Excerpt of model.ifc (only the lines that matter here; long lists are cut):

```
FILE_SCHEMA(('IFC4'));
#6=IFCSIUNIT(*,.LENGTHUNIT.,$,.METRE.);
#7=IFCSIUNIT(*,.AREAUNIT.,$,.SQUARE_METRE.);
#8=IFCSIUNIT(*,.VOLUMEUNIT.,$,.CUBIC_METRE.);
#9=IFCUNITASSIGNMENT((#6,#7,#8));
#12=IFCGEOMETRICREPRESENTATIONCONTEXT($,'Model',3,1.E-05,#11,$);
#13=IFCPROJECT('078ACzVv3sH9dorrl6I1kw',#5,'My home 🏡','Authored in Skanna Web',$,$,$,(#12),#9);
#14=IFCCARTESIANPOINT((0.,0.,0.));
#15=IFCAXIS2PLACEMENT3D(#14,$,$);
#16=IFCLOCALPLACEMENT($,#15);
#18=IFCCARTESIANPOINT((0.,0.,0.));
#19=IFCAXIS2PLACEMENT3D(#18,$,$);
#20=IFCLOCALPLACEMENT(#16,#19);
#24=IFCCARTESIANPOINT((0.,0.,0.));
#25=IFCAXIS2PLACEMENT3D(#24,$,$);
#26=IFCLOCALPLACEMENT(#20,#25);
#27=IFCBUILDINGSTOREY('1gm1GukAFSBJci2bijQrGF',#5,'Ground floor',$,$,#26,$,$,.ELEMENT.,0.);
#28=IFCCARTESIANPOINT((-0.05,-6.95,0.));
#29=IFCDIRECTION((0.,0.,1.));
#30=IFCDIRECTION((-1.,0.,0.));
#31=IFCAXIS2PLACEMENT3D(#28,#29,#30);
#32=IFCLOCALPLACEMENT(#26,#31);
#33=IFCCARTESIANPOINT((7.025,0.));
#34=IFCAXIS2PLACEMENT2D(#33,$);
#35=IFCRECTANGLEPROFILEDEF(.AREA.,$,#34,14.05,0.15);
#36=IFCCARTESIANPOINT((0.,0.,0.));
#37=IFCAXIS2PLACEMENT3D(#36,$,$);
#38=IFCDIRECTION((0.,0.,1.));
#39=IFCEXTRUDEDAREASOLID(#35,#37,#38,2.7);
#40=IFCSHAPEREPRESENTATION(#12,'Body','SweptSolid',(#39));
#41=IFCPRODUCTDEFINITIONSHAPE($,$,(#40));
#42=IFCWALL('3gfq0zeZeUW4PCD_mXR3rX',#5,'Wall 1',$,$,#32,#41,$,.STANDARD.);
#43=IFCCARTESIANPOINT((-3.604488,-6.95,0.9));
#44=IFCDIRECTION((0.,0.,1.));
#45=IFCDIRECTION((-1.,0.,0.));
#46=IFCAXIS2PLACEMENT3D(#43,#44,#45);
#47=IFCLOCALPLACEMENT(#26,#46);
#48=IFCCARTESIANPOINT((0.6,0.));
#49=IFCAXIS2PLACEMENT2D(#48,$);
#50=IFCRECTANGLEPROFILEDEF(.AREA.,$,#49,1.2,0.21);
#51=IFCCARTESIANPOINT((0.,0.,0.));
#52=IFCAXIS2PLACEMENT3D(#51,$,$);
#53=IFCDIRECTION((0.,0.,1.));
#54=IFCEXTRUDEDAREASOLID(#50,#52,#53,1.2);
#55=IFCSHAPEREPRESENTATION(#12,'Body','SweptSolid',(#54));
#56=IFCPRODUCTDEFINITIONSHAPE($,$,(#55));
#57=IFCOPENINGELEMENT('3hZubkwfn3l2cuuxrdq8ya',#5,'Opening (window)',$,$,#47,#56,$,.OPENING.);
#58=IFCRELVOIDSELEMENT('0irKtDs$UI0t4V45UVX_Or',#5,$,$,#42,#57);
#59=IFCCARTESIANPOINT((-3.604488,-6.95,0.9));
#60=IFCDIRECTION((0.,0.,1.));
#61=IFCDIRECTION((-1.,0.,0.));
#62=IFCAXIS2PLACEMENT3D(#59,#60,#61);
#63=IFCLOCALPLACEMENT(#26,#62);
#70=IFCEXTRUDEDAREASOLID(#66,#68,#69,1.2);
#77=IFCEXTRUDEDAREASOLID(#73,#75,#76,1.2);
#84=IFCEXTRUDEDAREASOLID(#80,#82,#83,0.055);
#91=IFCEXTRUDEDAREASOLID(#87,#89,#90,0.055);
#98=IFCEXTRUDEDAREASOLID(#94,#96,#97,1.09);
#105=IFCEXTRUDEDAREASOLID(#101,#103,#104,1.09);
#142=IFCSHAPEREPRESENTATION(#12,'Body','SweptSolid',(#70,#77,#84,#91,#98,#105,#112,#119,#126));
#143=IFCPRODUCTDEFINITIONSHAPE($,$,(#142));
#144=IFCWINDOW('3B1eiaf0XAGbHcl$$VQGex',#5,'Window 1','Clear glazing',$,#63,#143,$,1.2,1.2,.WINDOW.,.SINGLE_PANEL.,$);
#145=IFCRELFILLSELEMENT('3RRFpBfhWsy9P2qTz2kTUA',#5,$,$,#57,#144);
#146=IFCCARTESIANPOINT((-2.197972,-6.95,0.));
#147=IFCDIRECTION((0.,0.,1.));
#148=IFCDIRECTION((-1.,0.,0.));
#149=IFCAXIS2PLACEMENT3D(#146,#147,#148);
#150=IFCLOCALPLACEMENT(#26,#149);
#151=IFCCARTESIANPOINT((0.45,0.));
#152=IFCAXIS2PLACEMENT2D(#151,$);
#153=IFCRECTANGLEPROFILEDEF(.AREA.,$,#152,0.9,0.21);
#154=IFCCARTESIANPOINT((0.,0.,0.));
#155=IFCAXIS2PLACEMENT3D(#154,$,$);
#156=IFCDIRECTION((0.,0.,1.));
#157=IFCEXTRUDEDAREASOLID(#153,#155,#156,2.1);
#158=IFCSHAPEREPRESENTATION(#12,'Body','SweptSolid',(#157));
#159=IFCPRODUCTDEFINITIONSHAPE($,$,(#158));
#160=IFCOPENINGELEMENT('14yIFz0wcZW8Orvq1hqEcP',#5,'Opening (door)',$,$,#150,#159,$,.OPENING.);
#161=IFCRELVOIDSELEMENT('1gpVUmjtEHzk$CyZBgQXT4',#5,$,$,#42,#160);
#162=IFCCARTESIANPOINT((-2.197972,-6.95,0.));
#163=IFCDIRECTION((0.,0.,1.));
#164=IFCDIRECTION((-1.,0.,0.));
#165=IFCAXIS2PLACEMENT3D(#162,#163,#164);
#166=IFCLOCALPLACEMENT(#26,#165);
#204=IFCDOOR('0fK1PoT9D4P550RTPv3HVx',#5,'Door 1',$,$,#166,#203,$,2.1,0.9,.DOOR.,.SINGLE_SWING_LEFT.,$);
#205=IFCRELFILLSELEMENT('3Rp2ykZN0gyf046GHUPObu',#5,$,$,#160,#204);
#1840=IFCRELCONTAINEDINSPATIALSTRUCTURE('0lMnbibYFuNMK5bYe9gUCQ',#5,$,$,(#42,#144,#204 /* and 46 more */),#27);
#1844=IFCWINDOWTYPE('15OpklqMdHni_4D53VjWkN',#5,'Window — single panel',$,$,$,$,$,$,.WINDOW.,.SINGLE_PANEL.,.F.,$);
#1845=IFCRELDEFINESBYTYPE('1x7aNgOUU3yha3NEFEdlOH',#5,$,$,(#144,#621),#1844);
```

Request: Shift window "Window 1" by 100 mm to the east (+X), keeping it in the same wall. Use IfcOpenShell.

```python
import ifcopenshell
import ifcopenshell.api.geometry
import ifcopenshell.util.placement
import ifcopenshell.util.unit

model = ifcopenshell.open("model.ifc")
unit_scale = ifcopenshell.util.unit.calculate_unit_scale(model)

window = model.by_id(144)
opening = window.FillsVoids[0].RelatingOpeningElement
wall = opening.VoidsElements[0].RelatingBuildingElement

wall_matrix = ifcopenshell.util.placement.get_local_placement(wall.ObjectPlacement)
shift = wall_matrix[:3, 0] * -0.1 / unit_scale
before = ifcopenshell.util.placement.get_local_placement(window.ObjectPlacement)[:3, 3].copy()

# The window is not placed relative to its opening, so move both.
for product in (opening, window):
    matrix = ifcopenshell.util.placement.get_local_placement(product.ObjectPlacement)
    matrix[:3, 3] += shift
    ifcopenshell.api.geometry.edit_object_placement(model, product=product, matrix=matrix, is_si=False)

after = ifcopenshell.util.placement.get_local_placement(window.ObjectPlacement)[:3, 3]
print("window moved by", (after - before).round(3) + 0.0)

model.write("model_rev.ifc")
```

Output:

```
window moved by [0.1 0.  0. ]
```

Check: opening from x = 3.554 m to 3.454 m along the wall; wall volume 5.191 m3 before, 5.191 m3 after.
